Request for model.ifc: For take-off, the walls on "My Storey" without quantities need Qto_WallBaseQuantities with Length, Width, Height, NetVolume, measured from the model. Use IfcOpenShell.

First a look at what the model holds.

```python
import ifcopenshell
import ifcopenshell.util.element
import ifcopenshell.util.unit

model = ifcopenshell.open("model.ifc")
print(model.schema)
for unit_type in ("LENGTHUNIT", "AREAUNIT", "VOLUMEUNIT"):
    print(unit_type, ifcopenshell.util.unit.calculate_unit_scale(model, unit_type))
storey = next(s for s in model.by_type("IfcBuildingStorey") if s.Name == "My Storey")
walls = [e for e in ifcopenshell.util.element.get_decomposition(storey) if e.is_a("IfcWall")]
for e in sorted(walls, key=lambda e: e.id()):
    print(e.id(), e.is_a(), e.Name, list(ifcopenshell.util.element.get_psets(e, qtos_only=True)), sep=" | ")
```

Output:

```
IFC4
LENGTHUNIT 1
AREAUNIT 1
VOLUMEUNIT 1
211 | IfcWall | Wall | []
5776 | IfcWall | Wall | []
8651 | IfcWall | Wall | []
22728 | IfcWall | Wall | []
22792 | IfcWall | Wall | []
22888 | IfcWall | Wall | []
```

```python
import ifcopenshell
import ifcopenshell.api.pset
import ifcopenshell.geom
import ifcopenshell.util.element
import ifcopenshell.util.shape
import ifcopenshell.util.unit

model = ifcopenshell.open("model.ifc")
unit_scale = ifcopenshell.util.unit.calculate_unit_scale(model)
volume_scale = ifcopenshell.util.unit.calculate_unit_scale(model, "VOLUMEUNIT")
settings = ifcopenshell.geom.settings()

storey = next(s for s in model.by_type("IfcBuildingStorey") if s.Name == "My Storey")
walls = [e for e in ifcopenshell.util.element.get_decomposition(storey) if e.is_a("IfcWall")]

for e in sorted(walls, key=lambda e: e.id()):
    if ifcopenshell.util.element.get_psets(e, qtos_only=True, should_inherit=False):
        continue
    # Geometry comes back in metres, in the element's own axes.
    shape = ifcopenshell.geom.create_shape(settings, e)
    values = {
        "Length": ifcopenshell.util.shape.get_x(shape.geometry) / unit_scale,
        "Width": ifcopenshell.util.shape.get_y(shape.geometry) / unit_scale,
        "Height": ifcopenshell.util.shape.get_z(shape.geometry) / unit_scale,
        "NetVolume": ifcopenshell.util.shape.get_volume(shape.geometry) / volume_scale,
    }
    qto = ifcopenshell.api.pset.add_qto(model, product=e, name="Qto_WallBaseQuantities")
    ifcopenshell.api.pset.edit_qto(model, qto=qto, properties=values)
    print(e.id(), {k: round(v, 3) for k, v in values.items()})

model.write("model_v2.ifc")
```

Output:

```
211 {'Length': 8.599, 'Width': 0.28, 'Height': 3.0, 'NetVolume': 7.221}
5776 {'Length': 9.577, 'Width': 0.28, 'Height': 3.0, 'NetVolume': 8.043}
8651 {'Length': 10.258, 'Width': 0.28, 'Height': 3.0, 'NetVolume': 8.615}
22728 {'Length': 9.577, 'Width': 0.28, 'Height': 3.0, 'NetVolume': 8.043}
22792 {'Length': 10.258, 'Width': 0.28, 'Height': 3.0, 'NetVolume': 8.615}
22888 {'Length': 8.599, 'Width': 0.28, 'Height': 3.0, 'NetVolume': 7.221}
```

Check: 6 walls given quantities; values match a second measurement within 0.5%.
